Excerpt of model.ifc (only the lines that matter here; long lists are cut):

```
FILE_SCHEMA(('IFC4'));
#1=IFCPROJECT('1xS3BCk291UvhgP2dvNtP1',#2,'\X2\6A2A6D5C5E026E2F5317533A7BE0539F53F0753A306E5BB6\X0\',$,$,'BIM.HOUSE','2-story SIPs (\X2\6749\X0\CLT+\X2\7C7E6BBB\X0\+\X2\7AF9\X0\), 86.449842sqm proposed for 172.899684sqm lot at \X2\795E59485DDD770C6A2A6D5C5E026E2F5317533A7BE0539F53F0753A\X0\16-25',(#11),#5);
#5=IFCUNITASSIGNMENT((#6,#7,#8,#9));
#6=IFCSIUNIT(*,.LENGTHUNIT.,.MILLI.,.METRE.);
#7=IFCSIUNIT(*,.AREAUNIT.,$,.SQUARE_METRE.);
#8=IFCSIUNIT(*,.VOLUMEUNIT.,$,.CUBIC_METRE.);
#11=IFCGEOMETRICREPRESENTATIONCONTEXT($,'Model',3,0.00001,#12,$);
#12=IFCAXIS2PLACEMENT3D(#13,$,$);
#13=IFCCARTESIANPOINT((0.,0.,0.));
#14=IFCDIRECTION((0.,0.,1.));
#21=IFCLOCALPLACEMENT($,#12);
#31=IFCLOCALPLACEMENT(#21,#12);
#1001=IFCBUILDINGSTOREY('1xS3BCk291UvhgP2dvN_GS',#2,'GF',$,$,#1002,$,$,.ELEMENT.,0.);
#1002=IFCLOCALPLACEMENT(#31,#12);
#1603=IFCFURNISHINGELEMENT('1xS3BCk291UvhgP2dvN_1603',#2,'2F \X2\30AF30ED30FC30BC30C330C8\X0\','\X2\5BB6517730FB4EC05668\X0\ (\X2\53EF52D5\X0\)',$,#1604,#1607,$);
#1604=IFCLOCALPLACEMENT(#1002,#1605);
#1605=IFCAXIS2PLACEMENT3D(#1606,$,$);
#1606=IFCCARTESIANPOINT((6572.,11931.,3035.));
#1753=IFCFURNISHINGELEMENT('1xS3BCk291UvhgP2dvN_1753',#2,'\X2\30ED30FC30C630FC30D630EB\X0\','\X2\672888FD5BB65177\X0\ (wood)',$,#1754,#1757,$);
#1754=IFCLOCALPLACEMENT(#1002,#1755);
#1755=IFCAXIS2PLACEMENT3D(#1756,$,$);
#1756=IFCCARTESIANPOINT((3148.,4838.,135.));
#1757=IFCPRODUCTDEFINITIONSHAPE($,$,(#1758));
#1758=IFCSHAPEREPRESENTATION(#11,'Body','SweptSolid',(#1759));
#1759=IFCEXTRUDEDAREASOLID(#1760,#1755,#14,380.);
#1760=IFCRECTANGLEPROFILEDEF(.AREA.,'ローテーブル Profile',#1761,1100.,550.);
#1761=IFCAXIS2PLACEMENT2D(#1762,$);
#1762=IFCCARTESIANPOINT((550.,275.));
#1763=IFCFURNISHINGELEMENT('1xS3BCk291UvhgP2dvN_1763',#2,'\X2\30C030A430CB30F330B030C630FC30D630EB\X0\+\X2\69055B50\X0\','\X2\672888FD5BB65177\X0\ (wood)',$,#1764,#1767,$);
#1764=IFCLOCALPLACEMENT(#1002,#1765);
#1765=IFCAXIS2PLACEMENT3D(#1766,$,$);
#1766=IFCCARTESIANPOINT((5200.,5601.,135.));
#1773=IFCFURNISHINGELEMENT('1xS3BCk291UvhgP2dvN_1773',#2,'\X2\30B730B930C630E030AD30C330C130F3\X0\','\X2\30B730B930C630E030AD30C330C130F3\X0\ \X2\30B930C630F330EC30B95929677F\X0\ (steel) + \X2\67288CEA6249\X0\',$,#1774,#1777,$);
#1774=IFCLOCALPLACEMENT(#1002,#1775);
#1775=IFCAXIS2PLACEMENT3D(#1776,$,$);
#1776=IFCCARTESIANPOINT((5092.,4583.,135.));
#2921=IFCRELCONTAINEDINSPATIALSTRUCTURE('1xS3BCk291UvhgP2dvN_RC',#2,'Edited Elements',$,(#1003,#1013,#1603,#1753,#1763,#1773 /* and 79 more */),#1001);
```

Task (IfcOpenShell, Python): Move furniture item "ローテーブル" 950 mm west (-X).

```python
import ifcopenshell
import ifcopenshell.api.geometry
import ifcopenshell.util.placement

model = ifcopenshell.open("model.ifc")

item = model.by_guid("1xS3BCk291UvhgP2dvN_1753")
matrix = ifcopenshell.util.placement.get_local_placement(item.ObjectPlacement)
matrix[0, 3] -= 950.0
ifcopenshell.api.geometry.edit_object_placement(model, product=item, matrix=matrix, is_si=False)

print(ifcopenshell.util.placement.get_local_placement(item.ObjectPlacement).round(3) + 0.0)

model.write("model_v2.ifc")
```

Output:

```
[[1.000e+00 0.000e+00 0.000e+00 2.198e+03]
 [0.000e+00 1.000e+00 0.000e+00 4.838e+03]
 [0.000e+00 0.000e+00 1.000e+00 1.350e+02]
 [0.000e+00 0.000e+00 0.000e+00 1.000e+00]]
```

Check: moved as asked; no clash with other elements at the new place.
